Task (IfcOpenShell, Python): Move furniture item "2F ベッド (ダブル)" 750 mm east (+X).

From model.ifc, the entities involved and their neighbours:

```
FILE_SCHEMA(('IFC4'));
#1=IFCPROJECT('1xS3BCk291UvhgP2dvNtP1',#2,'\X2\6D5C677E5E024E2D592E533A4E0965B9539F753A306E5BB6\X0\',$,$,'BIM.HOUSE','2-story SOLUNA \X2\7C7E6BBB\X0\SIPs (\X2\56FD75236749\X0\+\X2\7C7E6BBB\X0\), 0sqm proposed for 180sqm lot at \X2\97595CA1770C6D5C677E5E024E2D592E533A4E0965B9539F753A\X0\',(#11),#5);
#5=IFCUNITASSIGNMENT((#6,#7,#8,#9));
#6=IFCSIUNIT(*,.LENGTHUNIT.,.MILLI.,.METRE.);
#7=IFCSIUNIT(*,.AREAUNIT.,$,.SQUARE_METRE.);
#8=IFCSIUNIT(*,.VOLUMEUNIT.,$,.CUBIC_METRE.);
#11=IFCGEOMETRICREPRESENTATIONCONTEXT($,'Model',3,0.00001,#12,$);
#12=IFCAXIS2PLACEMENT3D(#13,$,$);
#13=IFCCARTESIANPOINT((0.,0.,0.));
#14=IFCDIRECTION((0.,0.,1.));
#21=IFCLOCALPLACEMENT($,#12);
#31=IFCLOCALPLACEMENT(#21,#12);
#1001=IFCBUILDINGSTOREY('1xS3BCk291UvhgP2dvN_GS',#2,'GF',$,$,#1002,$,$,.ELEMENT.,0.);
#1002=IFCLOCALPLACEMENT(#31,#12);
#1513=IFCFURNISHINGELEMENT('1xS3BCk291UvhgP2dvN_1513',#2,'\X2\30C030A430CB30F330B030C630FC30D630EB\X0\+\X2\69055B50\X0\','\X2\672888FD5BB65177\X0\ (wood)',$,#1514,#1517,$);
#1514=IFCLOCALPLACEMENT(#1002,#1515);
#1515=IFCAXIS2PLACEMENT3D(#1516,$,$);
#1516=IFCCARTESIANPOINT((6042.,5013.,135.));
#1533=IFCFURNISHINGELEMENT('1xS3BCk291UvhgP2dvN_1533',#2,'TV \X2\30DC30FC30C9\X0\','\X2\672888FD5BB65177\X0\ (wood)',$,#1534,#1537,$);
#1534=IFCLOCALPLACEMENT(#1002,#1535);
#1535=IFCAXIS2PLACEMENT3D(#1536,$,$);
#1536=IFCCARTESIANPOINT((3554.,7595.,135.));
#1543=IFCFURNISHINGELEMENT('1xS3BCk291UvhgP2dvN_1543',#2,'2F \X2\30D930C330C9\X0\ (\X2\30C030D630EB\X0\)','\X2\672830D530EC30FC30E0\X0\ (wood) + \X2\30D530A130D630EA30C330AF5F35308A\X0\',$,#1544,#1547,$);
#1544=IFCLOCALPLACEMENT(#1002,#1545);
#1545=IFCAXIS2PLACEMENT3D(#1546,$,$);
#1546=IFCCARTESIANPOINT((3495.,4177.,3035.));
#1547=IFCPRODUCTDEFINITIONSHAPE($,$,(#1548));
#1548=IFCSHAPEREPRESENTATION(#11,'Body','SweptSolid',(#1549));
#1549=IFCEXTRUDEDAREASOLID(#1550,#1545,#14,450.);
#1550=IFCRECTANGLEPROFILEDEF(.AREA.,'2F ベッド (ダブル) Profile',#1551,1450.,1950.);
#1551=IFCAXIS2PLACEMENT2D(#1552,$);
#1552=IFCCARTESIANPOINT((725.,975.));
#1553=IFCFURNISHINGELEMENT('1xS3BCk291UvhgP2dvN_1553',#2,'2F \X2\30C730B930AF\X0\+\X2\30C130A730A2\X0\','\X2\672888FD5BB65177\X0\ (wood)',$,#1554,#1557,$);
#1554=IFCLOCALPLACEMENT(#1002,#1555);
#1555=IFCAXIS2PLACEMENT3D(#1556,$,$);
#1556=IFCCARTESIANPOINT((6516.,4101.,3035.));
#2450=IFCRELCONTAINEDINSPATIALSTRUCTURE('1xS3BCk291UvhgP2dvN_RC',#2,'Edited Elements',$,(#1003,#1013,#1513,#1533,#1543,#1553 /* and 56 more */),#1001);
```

```python
import ifcopenshell
import ifcopenshell.api.geometry
import ifcopenshell.util.placement

model = ifcopenshell.open("model.ifc")

item = model.by_guid("1xS3BCk291UvhgP2dvN_1543")
matrix = ifcopenshell.util.placement.get_local_placement(item.ObjectPlacement)
matrix[0, 3] += 750.0
ifcopenshell.api.geometry.edit_object_placement(model, product=item, matrix=matrix, is_si=False)

print(ifcopenshell.util.placement.get_local_placement(item.ObjectPlacement).round(3) + 0.0)

model.write("model_rev.ifc")
```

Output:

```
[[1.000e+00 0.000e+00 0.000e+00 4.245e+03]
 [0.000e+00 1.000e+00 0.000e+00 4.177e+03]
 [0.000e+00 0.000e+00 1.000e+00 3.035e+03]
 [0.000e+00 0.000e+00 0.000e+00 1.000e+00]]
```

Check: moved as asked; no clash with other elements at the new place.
